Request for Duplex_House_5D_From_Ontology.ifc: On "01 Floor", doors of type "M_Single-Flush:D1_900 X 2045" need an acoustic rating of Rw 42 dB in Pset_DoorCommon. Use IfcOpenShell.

First a look at what the model holds.

```python
import ifcopenshell
import ifcopenshell.util.element

model = ifcopenshell.open("Duplex_House_5D_From_Ontology.ifc")
print(model.schema)
storey = next(s for s in model.by_type("IfcBuildingStorey") if s.Name == "01 Floor")
doors = [e for e in ifcopenshell.util.element.get_decomposition(storey) if e.is_a("IfcDoor")]
seen = {}
for e in doors:
    element_type = ifcopenshell.util.element.get_type(e)
    key = (element_type.Name if element_type != e and element_type else None, ifcopenshell.util.element.get_pset(e, "Pset_DoorCommon", "AcousticRating"))
    seen[key] = seen.get(key, 0) + 1
for (name, value), count in sorted(seen.items(), key=str):
    print(count, "x", name, "|", value)
```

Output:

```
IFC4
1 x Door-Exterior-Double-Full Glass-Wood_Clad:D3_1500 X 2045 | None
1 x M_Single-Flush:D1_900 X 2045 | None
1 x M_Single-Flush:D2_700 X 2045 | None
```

```python
import ifcopenshell
import ifcopenshell.api.pset
import ifcopenshell.util.element

model = ifcopenshell.open("Duplex_House_5D_From_Ontology.ifc")

storey = next(s for s in model.by_type("IfcBuildingStorey") if s.Name == "01 Floor")
doors = [e for e in ifcopenshell.util.element.get_decomposition(storey) if e.is_a("IfcDoor")]

count = 0
for e in doors:
    element_type = ifcopenshell.util.element.get_type(e)
    if element_type in (None, e) or element_type.Name != "M_Single-Flush:D1_900 X 2045":
        continue
    # add_pset returns the element's existing set when there is one.
    pset = ifcopenshell.api.pset.add_pset(model, product=e, name="Pset_DoorCommon")
    ifcopenshell.api.pset.edit_pset(model, pset=pset, properties={"AcousticRating": "Rw 42 dB"})
    count += 1

print(count, "doors updated")

model.write("Duplex_House_5D_From_Ontology_rev.ifc")
```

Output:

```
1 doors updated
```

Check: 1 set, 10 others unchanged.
